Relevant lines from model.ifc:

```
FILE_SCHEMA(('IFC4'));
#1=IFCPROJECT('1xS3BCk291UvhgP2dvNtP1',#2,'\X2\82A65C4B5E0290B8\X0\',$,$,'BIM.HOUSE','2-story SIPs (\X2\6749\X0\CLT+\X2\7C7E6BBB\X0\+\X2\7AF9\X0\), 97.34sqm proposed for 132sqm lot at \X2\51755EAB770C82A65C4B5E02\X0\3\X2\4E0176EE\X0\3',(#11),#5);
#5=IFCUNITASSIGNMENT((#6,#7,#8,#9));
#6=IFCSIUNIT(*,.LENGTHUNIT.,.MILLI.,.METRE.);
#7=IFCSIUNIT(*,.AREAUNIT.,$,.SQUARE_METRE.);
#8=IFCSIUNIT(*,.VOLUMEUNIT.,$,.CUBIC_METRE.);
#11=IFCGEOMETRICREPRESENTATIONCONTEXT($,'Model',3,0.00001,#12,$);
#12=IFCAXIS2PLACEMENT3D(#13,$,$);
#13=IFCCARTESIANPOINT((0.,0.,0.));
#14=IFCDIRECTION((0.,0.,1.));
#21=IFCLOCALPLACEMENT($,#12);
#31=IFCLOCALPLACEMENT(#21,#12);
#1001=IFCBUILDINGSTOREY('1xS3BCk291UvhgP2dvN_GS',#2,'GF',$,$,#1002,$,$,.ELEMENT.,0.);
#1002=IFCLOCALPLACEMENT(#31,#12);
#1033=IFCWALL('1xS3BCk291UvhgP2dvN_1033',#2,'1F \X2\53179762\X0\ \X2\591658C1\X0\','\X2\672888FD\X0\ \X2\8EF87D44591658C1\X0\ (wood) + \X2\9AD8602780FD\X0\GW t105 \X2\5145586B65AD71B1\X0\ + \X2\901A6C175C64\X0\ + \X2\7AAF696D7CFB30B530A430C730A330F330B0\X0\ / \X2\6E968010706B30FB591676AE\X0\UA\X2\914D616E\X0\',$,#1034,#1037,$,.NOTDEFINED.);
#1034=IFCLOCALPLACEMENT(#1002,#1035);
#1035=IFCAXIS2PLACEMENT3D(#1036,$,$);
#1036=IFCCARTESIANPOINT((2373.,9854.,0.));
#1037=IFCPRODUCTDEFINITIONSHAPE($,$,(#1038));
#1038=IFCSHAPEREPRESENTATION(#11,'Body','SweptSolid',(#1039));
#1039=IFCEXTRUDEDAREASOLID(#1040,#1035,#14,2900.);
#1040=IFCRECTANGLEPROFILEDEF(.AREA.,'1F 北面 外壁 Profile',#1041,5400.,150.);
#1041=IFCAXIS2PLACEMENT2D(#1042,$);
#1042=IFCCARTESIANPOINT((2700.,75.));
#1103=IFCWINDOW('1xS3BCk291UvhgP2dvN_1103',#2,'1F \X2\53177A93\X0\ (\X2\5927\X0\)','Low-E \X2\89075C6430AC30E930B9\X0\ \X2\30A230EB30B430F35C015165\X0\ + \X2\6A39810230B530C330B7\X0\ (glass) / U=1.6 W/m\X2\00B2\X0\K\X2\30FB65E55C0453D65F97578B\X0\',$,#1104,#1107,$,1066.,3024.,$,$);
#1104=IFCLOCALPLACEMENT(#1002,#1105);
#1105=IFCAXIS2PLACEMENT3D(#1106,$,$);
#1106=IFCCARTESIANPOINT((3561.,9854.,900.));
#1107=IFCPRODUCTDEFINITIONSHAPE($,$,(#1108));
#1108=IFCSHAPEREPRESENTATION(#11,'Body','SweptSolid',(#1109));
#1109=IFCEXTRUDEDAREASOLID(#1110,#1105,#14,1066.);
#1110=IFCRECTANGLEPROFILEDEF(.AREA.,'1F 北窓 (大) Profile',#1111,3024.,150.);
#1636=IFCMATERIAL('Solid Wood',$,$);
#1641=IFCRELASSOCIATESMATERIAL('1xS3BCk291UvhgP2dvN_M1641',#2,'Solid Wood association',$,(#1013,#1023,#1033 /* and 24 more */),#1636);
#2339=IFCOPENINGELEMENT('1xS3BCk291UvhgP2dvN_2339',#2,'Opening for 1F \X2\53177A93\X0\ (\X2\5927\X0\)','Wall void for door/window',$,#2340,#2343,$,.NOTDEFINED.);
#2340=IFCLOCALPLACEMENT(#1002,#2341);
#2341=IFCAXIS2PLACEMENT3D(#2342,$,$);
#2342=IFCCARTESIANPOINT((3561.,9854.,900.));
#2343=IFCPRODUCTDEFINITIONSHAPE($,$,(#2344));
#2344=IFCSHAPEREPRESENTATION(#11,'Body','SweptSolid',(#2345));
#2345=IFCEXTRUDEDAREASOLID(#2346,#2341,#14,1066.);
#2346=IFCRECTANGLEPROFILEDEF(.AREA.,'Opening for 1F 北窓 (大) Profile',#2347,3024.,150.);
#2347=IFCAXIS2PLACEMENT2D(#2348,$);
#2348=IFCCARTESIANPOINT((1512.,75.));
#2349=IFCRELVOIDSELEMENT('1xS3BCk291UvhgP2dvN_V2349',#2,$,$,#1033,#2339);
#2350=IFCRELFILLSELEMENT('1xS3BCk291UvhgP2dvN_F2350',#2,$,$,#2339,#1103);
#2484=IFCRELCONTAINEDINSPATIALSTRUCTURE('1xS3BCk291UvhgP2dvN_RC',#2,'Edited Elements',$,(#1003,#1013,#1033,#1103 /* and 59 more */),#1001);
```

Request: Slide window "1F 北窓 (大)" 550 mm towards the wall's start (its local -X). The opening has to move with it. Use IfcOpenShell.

```python
import ifcopenshell
import ifcopenshell.api.geometry
import ifcopenshell.util.placement

model = ifcopenshell.open("model.ifc")

window = model.by_guid("1xS3BCk291UvhgP2dvN_1103")
opening = window.FillsVoids[0].RelatingOpeningElement
wall = opening.VoidsElements[0].RelatingBuildingElement

wall_matrix = ifcopenshell.util.placement.get_local_placement(wall.ObjectPlacement)
shift = wall_matrix[:3, 0] * -550.0
before = ifcopenshell.util.placement.get_local_placement(window.ObjectPlacement)[:3, 3].copy()

# The window is not placed relative to its opening, so move both.
for product in (opening, window):
    matrix = ifcopenshell.util.placement.get_local_placement(product.ObjectPlacement)
    matrix[:3, 3] += shift
    ifcopenshell.api.geometry.edit_object_placement(model, product=product, matrix=matrix, is_si=False)

after = ifcopenshell.util.placement.get_local_placement(window.ObjectPlacement)[:3, 3]
print("window moved by", (after - before).round(3) + 0.0)

model.write("model_updated.ifc")
```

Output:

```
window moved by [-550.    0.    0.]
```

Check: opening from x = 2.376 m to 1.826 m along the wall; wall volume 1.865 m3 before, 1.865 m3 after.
